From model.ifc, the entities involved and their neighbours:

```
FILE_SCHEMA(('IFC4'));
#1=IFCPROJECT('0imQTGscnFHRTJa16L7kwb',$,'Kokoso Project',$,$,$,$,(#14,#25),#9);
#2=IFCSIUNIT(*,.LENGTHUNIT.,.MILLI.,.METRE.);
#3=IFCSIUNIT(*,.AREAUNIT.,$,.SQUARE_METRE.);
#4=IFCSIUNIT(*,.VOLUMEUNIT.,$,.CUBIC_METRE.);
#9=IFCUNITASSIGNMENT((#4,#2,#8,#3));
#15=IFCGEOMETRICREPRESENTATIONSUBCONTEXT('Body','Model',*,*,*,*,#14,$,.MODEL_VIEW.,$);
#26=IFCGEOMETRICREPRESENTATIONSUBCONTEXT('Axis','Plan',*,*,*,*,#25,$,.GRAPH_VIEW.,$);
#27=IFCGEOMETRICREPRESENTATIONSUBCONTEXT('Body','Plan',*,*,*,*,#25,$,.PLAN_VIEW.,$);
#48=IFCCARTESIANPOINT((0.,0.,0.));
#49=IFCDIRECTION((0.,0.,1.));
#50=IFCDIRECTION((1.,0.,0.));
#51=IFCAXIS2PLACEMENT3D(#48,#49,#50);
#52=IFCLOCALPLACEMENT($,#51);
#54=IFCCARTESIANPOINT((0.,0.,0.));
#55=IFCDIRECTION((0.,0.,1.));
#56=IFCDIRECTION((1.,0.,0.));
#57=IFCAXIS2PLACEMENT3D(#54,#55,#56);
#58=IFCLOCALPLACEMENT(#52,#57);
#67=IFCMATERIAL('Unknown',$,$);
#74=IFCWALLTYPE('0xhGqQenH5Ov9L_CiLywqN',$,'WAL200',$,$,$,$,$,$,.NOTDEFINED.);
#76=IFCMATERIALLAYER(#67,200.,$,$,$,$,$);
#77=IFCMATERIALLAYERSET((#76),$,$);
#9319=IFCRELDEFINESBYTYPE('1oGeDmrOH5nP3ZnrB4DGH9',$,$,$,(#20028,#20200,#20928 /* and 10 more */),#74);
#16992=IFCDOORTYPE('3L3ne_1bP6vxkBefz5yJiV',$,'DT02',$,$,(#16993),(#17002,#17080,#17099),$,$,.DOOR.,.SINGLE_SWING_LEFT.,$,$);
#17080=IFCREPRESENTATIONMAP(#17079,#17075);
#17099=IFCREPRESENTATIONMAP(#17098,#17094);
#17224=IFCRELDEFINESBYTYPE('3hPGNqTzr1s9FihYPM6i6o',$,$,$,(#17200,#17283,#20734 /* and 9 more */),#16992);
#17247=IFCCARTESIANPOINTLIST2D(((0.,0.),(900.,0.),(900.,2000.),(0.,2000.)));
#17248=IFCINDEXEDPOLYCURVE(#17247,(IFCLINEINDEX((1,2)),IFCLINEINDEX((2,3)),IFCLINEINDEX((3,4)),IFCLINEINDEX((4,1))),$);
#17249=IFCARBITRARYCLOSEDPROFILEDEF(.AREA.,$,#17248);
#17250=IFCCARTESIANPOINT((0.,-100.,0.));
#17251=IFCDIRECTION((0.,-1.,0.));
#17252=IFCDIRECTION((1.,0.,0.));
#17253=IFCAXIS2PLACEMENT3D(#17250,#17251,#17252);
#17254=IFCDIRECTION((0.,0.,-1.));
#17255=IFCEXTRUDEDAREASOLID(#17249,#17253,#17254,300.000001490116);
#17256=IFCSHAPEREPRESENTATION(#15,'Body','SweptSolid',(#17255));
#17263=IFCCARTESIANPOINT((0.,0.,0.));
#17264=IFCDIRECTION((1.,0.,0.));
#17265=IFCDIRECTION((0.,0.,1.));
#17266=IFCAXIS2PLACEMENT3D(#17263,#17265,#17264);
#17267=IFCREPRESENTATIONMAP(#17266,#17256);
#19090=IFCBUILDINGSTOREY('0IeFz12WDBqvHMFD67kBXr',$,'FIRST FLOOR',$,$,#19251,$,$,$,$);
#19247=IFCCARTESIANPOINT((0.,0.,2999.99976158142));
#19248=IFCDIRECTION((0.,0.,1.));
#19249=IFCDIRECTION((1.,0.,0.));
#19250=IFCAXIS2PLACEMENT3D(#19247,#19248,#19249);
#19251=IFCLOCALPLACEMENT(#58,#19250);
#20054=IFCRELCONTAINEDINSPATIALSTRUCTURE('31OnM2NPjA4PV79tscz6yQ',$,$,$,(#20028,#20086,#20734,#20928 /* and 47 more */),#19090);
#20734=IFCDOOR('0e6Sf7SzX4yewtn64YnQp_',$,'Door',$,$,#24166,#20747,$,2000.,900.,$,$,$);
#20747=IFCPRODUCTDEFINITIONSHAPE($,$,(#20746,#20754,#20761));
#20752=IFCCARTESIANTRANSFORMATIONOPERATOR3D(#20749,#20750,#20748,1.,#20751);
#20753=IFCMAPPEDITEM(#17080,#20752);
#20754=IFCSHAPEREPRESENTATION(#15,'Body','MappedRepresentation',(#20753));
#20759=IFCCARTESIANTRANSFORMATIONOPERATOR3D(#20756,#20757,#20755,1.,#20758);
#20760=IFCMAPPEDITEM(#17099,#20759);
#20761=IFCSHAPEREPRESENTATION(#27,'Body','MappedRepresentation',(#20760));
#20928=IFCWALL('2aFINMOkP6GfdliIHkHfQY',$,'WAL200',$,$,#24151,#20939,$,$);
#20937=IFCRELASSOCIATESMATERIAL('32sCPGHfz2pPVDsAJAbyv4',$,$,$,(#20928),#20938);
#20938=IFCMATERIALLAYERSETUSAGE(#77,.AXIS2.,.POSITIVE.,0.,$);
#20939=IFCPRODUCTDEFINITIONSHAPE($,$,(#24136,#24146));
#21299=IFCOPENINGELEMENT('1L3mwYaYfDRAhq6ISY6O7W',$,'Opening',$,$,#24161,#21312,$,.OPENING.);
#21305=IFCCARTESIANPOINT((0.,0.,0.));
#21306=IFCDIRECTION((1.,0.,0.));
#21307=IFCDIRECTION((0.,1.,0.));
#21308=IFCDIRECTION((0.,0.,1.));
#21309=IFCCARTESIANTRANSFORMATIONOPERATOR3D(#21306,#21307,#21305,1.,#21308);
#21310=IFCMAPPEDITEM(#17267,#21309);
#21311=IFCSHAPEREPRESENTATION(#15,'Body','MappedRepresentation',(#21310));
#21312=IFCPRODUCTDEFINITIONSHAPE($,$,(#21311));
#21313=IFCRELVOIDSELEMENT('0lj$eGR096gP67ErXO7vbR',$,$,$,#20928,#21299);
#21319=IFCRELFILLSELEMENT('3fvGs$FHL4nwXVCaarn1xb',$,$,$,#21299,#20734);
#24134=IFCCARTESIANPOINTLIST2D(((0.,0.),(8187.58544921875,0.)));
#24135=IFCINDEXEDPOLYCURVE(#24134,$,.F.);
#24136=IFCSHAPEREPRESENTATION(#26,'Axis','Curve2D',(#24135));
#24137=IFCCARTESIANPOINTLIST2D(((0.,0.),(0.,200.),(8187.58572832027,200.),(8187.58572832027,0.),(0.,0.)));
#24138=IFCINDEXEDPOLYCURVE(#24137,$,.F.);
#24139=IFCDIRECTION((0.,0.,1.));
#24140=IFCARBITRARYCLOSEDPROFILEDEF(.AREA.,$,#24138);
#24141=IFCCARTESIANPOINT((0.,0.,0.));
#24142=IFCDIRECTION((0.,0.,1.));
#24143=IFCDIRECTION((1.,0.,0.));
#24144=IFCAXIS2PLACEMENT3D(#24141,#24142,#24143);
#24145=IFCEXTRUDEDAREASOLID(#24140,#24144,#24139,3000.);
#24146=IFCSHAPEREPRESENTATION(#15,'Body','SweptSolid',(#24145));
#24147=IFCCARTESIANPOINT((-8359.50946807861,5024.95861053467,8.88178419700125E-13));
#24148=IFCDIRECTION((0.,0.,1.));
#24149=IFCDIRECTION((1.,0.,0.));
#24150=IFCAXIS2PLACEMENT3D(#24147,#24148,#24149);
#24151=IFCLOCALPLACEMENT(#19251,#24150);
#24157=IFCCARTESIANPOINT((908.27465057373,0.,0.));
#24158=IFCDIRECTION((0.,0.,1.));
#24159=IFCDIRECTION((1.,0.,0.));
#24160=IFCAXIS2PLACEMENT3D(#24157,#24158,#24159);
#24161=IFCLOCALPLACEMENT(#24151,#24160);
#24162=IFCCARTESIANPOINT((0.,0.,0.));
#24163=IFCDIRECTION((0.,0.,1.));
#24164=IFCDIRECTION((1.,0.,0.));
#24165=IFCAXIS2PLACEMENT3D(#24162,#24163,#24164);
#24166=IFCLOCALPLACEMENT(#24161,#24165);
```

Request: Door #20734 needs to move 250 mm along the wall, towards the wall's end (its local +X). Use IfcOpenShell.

```python
import ifcopenshell
import ifcopenshell.api.geometry
import ifcopenshell.util.placement

model = ifcopenshell.open("model.ifc")

door = model.by_guid("0e6Sf7SzX4yewtn64YnQp_")
opening = door.FillsVoids[0].RelatingOpeningElement
wall = opening.VoidsElements[0].RelatingBuildingElement

wall_matrix = ifcopenshell.util.placement.get_local_placement(wall.ObjectPlacement)
shift = wall_matrix[:3, 0] * 250.0
before = ifcopenshell.util.placement.get_local_placement(door.ObjectPlacement)[:3, 3].copy()

# The door is placed relative to its opening, so it follows when the opening moves.
matrix = ifcopenshell.util.placement.get_local_placement(opening.ObjectPlacement)
matrix[:3, 3] += shift
ifcopenshell.api.geometry.edit_object_placement(
    model, product=opening, matrix=matrix, is_si=False, should_transform_children=True
)

after = ifcopenshell.util.placement.get_local_placement(door.ObjectPlacement)[:3, 3]
print("door moved by", (after - before).round(3) + 0.0)

model.write("model_v2.ifc")
```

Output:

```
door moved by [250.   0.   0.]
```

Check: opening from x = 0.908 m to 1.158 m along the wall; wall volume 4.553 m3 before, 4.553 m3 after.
